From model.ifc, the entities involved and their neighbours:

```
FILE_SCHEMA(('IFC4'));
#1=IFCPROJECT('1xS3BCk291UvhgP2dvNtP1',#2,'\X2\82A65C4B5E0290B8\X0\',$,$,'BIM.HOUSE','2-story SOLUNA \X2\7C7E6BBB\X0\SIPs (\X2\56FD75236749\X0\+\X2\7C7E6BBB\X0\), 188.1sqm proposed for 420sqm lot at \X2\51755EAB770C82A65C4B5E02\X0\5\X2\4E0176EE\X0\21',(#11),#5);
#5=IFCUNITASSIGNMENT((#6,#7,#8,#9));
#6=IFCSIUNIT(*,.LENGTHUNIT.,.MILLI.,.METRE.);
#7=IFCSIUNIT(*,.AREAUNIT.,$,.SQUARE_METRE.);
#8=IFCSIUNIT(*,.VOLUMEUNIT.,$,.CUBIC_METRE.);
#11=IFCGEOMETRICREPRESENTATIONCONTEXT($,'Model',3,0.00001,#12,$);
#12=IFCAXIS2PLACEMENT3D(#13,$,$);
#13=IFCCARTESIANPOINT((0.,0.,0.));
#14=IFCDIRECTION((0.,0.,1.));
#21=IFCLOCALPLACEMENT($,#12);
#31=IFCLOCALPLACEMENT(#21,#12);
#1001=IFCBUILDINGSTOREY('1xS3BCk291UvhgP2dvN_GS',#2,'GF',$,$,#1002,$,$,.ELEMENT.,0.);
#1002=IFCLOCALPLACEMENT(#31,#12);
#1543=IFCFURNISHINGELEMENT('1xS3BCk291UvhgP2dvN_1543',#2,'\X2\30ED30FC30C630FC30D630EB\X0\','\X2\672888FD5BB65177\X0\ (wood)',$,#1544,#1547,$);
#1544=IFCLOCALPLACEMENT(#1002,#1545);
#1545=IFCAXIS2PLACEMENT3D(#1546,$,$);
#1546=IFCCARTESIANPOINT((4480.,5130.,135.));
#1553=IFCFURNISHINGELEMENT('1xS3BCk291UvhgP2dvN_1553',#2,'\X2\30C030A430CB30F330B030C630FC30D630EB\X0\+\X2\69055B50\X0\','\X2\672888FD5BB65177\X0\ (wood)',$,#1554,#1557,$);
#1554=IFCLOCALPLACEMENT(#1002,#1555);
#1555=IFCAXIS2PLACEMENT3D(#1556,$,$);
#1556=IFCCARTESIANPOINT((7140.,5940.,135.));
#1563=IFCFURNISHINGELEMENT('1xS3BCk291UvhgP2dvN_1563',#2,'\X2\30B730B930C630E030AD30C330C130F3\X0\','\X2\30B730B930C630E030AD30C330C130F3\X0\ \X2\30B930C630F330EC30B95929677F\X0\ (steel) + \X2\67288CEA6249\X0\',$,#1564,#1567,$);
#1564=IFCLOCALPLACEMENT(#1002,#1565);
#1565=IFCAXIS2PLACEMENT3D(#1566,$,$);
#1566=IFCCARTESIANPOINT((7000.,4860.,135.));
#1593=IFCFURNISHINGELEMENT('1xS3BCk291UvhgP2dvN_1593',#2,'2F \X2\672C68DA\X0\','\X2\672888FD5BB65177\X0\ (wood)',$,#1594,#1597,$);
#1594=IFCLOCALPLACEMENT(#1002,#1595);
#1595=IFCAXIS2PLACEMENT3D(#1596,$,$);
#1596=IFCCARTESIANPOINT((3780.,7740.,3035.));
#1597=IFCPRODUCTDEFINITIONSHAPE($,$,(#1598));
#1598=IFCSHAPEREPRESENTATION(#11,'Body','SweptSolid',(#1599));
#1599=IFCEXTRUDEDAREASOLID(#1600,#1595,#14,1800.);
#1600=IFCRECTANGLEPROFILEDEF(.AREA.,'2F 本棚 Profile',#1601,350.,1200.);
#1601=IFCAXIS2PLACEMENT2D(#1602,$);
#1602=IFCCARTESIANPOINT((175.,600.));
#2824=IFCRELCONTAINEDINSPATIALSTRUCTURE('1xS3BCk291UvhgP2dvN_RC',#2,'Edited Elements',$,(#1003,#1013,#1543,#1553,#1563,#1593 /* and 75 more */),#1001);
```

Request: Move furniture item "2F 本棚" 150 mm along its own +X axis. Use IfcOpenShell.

```python
import ifcopenshell
import ifcopenshell.api.geometry
import ifcopenshell.util.placement

model = ifcopenshell.open("model.ifc")

item = model.by_guid("1xS3BCk291UvhgP2dvN_1593")
matrix = ifcopenshell.util.placement.get_local_placement(item.ObjectPlacement)
matrix[:3, 3] += matrix[:3, 0] * 150.0
ifcopenshell.api.geometry.edit_object_placement(model, product=item, matrix=matrix, is_si=False)

print(ifcopenshell.util.placement.get_local_placement(item.ObjectPlacement).round(3) + 0.0)

model.write("model-out.ifc")
```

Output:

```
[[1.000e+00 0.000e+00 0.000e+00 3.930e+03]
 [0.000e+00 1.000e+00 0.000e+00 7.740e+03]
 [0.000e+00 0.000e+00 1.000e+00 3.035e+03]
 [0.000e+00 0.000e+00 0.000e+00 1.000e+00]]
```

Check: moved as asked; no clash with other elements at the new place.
